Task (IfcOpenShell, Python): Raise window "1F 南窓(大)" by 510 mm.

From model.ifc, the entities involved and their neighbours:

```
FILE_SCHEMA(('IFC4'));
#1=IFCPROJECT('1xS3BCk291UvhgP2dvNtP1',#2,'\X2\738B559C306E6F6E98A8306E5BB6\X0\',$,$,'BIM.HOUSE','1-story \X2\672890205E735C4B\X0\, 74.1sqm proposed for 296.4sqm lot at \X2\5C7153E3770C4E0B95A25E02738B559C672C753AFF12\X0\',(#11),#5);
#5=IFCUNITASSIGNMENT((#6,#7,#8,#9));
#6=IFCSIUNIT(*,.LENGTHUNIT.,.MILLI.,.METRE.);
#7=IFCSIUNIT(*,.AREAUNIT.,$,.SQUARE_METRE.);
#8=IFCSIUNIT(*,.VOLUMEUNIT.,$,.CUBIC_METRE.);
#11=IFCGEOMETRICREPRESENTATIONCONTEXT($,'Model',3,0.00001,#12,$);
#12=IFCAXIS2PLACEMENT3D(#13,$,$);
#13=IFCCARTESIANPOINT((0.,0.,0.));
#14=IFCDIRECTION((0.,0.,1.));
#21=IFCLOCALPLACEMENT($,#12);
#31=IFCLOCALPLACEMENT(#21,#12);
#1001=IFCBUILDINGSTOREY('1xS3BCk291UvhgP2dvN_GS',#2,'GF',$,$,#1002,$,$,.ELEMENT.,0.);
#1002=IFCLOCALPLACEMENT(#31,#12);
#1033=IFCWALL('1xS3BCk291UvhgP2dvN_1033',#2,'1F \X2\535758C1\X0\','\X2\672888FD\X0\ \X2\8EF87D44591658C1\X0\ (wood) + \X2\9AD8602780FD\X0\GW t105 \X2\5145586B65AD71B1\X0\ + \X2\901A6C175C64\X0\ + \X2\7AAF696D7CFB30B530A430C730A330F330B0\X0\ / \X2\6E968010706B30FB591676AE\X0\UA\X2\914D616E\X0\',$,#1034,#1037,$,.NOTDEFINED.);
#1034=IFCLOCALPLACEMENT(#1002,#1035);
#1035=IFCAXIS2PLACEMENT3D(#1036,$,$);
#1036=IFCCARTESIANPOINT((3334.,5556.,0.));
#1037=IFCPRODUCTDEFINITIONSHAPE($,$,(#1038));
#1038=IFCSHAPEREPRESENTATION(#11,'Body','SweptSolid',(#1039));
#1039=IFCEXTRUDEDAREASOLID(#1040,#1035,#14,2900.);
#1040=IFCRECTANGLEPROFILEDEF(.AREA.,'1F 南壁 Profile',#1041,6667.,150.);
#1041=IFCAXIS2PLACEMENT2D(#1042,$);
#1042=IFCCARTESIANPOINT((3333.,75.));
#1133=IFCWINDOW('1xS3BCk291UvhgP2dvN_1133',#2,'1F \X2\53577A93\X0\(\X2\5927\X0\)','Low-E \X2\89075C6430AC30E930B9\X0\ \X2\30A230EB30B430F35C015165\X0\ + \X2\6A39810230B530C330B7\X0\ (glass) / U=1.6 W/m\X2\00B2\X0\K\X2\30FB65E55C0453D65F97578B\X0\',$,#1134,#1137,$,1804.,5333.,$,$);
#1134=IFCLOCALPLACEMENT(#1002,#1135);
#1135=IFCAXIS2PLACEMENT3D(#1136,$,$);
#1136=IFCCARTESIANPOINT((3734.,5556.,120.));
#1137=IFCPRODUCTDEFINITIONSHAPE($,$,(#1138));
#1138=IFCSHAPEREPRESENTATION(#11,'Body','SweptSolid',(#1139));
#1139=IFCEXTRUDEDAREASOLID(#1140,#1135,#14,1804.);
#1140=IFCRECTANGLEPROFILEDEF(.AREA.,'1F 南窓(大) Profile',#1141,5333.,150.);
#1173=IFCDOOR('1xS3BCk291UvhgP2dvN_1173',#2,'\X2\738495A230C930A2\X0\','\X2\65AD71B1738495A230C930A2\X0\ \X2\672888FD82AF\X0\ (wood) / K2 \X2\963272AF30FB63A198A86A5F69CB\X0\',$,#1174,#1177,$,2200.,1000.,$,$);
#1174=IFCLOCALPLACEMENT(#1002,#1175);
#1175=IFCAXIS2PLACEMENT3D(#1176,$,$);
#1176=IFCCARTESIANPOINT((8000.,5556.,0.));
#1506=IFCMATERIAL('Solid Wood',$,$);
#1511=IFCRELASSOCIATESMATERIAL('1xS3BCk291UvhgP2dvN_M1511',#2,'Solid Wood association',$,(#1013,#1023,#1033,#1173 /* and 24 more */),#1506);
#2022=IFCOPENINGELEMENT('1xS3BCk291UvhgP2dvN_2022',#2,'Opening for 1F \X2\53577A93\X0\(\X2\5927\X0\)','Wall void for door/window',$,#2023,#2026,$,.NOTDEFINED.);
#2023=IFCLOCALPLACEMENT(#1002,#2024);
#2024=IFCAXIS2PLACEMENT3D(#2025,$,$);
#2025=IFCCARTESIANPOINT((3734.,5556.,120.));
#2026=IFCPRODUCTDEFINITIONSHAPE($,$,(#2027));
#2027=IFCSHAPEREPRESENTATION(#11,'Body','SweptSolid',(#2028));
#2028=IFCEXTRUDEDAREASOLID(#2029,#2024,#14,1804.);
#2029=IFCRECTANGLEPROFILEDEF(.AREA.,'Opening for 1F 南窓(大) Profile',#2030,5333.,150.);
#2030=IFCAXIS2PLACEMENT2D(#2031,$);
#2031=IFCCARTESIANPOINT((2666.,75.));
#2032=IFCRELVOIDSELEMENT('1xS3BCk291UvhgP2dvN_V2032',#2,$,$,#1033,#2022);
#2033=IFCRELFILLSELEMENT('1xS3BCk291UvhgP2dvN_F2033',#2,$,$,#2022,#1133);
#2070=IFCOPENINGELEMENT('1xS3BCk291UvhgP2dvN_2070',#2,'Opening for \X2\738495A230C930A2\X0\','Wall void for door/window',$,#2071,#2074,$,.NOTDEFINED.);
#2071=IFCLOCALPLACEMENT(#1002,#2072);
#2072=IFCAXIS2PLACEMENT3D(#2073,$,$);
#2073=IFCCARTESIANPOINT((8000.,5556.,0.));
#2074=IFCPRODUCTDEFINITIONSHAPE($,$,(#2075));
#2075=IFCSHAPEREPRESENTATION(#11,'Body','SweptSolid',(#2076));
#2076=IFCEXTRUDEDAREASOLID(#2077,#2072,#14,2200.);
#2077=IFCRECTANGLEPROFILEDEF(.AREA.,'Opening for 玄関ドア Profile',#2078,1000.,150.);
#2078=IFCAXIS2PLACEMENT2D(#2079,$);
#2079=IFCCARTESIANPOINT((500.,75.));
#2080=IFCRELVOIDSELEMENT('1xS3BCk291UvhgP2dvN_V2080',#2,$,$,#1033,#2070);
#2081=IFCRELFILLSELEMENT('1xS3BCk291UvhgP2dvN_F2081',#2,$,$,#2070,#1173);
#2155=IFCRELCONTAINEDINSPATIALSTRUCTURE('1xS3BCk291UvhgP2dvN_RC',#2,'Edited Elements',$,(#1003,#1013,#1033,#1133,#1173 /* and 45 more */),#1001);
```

```python
import numpy as np
import ifcopenshell
import ifcopenshell.api.geometry
import ifcopenshell.util.placement
import ifcopenshell.util.unit

model = ifcopenshell.open("model.ifc")
unit_scale = ifcopenshell.util.unit.calculate_unit_scale(model)

window = model.by_guid("1xS3BCk291UvhgP2dvN_1133")
opening = window.FillsVoids[0].RelatingOpeningElement
dz = 510.0

shift = np.array([0.0, 0.0, dz])
# The window is not placed relative to its opening, so move both.
for product in (opening, window):
    matrix = ifcopenshell.util.placement.get_local_placement(product.ObjectPlacement)
    matrix[:3, 3] += shift
    ifcopenshell.api.geometry.edit_object_placement(model, product=product, matrix=matrix, is_si=False)

print(f"moved by {dz * unit_scale:+.3f} m")

model.write("model-out.ifc")
```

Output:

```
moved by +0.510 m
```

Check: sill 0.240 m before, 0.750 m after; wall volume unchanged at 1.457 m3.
